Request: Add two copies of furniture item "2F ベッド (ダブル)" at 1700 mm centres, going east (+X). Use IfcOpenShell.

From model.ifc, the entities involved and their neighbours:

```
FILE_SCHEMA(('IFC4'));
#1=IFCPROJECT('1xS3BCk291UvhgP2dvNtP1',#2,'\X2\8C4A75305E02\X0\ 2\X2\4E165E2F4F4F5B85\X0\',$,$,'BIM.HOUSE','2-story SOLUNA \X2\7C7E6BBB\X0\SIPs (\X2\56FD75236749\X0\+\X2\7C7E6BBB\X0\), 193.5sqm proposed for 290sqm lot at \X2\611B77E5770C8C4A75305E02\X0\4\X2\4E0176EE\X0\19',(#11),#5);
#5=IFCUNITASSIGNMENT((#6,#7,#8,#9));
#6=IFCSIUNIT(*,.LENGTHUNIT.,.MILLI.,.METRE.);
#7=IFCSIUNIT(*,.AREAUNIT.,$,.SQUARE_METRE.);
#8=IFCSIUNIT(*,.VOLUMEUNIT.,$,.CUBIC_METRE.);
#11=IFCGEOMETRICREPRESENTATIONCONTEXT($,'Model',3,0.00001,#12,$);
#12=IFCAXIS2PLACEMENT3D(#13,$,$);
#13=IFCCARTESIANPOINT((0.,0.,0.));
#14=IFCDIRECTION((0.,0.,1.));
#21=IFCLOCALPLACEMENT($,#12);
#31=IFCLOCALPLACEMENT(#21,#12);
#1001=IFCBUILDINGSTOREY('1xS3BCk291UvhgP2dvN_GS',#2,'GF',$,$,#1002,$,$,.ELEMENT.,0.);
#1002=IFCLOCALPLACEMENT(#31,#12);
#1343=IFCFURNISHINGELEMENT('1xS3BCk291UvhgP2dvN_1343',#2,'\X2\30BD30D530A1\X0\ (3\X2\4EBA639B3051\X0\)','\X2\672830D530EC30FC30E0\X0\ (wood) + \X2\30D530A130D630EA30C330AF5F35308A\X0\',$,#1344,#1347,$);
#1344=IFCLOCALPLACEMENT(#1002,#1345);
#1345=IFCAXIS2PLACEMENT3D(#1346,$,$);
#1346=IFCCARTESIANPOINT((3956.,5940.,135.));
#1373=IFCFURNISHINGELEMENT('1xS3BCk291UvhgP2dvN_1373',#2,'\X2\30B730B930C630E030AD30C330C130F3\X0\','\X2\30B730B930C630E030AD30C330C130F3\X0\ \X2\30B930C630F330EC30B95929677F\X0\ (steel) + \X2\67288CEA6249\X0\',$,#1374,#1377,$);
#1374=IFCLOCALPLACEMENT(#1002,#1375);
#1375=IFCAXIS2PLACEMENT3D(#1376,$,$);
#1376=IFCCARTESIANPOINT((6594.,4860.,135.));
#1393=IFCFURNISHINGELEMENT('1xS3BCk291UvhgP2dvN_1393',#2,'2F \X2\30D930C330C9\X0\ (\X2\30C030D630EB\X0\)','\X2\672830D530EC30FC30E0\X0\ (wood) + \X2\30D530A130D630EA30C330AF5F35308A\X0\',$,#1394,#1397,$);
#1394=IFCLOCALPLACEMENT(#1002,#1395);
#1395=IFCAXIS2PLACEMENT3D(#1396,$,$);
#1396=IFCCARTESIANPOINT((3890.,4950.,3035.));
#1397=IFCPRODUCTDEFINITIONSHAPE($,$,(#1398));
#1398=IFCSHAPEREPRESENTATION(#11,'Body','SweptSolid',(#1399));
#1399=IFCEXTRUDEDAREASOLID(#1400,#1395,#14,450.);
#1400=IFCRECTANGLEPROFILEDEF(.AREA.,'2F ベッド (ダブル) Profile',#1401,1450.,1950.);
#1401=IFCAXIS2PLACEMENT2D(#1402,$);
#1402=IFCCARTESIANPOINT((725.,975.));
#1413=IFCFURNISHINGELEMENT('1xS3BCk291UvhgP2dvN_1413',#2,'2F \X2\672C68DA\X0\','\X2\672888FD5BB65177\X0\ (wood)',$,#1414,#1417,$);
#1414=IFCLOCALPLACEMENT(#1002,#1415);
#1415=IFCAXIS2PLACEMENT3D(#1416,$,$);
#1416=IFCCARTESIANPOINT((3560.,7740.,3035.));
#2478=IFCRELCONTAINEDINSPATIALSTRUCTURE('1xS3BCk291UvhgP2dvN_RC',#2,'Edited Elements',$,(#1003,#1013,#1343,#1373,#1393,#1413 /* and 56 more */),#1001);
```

```python
import numpy as np
import ifcopenshell
import ifcopenshell.api.geometry
import ifcopenshell.api.root
import ifcopenshell.util.element
import ifcopenshell.util.placement
import ifcopenshell.util.unit

model = ifcopenshell.open("model.ifc")
unit_scale = ifcopenshell.util.unit.calculate_unit_scale(model)


def reuse_history(source, copy):
    """copy_class also copies each property set's owner history, people and application; keep the originals."""
    for rel in copy.IsDefinedBy:
        if rel.is_a("IfcRelDefinesByProperties") and (history := rel.RelatingPropertyDefinition.OwnerHistory):
            rel.RelatingPropertyDefinition.OwnerHistory = source.OwnerHistory
            ifcopenshell.util.element.remove_deep2(model, history)


source = model.by_guid("1xS3BCk291UvhgP2dvN_1393")
base = ifcopenshell.util.placement.get_local_placement(source.ObjectPlacement)
step = np.array([1.0, 0.0, 0.0]) * 1.7 / unit_scale

for i in range(1, 3):
    copy = ifcopenshell.api.root.copy_class(model, product=source)
    copy.Representation = ifcopenshell.util.element.copy_deep(
        model, source.Representation, exclude=["IfcGeometricRepresentationContext", "IfcRepresentationMap"]
    )
    reuse_history(source, copy)
    matrix = base.copy()
    matrix[:3, 3] += i * step
    print("added at", matrix[:3, 3].round(3) + 0.0)
    ifcopenshell.api.geometry.edit_object_placement(model, product=copy, matrix=matrix, is_si=False)

model.write("model-out.ifc")
```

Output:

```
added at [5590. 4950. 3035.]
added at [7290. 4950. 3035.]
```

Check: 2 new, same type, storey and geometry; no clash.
